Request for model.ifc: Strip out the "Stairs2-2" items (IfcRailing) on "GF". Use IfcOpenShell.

First a look at what the model holds.

```python
import ifcopenshell
import ifcopenshell.util.element

model = ifcopenshell.open("model.ifc")
print(model.schema)
storey = next(s for s in model.by_type("IfcBuildingStorey") if s.Name == "GF")
railings = [e for e in ifcopenshell.util.element.get_decomposition(storey) if e.is_a("IfcRailing")]
seen = {}
for e in railings:
    element_type = ifcopenshell.util.element.get_type(e)
    name = element_type.Name if element_type not in (None, e) else None
    seen[name] = seen.get(name, 0) + 1
for name, count in sorted(seen.items(), key=str):
    print(count, "x", name)
```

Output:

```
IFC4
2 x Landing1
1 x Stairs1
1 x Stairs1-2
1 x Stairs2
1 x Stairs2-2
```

```python
import ifcopenshell
import ifcopenshell.api.root
import ifcopenshell.util.element

model = ifcopenshell.open("model.ifc")

storey = next(s for s in model.by_type("IfcBuildingStorey") if s.Name == "GF")
railings = [e for e in ifcopenshell.util.element.get_decomposition(storey) if e.is_a("IfcRailing")]
targets = [e for e in railings if (t := ifcopenshell.util.element.get_type(e)) not in (None, e) and t.Name == "Stairs2-2"]

for e in targets:
    ifcopenshell.api.root.remove_product(model, product=e)
print(len(targets), "removed")

model.write("model_updated.ifc")
```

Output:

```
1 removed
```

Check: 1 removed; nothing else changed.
